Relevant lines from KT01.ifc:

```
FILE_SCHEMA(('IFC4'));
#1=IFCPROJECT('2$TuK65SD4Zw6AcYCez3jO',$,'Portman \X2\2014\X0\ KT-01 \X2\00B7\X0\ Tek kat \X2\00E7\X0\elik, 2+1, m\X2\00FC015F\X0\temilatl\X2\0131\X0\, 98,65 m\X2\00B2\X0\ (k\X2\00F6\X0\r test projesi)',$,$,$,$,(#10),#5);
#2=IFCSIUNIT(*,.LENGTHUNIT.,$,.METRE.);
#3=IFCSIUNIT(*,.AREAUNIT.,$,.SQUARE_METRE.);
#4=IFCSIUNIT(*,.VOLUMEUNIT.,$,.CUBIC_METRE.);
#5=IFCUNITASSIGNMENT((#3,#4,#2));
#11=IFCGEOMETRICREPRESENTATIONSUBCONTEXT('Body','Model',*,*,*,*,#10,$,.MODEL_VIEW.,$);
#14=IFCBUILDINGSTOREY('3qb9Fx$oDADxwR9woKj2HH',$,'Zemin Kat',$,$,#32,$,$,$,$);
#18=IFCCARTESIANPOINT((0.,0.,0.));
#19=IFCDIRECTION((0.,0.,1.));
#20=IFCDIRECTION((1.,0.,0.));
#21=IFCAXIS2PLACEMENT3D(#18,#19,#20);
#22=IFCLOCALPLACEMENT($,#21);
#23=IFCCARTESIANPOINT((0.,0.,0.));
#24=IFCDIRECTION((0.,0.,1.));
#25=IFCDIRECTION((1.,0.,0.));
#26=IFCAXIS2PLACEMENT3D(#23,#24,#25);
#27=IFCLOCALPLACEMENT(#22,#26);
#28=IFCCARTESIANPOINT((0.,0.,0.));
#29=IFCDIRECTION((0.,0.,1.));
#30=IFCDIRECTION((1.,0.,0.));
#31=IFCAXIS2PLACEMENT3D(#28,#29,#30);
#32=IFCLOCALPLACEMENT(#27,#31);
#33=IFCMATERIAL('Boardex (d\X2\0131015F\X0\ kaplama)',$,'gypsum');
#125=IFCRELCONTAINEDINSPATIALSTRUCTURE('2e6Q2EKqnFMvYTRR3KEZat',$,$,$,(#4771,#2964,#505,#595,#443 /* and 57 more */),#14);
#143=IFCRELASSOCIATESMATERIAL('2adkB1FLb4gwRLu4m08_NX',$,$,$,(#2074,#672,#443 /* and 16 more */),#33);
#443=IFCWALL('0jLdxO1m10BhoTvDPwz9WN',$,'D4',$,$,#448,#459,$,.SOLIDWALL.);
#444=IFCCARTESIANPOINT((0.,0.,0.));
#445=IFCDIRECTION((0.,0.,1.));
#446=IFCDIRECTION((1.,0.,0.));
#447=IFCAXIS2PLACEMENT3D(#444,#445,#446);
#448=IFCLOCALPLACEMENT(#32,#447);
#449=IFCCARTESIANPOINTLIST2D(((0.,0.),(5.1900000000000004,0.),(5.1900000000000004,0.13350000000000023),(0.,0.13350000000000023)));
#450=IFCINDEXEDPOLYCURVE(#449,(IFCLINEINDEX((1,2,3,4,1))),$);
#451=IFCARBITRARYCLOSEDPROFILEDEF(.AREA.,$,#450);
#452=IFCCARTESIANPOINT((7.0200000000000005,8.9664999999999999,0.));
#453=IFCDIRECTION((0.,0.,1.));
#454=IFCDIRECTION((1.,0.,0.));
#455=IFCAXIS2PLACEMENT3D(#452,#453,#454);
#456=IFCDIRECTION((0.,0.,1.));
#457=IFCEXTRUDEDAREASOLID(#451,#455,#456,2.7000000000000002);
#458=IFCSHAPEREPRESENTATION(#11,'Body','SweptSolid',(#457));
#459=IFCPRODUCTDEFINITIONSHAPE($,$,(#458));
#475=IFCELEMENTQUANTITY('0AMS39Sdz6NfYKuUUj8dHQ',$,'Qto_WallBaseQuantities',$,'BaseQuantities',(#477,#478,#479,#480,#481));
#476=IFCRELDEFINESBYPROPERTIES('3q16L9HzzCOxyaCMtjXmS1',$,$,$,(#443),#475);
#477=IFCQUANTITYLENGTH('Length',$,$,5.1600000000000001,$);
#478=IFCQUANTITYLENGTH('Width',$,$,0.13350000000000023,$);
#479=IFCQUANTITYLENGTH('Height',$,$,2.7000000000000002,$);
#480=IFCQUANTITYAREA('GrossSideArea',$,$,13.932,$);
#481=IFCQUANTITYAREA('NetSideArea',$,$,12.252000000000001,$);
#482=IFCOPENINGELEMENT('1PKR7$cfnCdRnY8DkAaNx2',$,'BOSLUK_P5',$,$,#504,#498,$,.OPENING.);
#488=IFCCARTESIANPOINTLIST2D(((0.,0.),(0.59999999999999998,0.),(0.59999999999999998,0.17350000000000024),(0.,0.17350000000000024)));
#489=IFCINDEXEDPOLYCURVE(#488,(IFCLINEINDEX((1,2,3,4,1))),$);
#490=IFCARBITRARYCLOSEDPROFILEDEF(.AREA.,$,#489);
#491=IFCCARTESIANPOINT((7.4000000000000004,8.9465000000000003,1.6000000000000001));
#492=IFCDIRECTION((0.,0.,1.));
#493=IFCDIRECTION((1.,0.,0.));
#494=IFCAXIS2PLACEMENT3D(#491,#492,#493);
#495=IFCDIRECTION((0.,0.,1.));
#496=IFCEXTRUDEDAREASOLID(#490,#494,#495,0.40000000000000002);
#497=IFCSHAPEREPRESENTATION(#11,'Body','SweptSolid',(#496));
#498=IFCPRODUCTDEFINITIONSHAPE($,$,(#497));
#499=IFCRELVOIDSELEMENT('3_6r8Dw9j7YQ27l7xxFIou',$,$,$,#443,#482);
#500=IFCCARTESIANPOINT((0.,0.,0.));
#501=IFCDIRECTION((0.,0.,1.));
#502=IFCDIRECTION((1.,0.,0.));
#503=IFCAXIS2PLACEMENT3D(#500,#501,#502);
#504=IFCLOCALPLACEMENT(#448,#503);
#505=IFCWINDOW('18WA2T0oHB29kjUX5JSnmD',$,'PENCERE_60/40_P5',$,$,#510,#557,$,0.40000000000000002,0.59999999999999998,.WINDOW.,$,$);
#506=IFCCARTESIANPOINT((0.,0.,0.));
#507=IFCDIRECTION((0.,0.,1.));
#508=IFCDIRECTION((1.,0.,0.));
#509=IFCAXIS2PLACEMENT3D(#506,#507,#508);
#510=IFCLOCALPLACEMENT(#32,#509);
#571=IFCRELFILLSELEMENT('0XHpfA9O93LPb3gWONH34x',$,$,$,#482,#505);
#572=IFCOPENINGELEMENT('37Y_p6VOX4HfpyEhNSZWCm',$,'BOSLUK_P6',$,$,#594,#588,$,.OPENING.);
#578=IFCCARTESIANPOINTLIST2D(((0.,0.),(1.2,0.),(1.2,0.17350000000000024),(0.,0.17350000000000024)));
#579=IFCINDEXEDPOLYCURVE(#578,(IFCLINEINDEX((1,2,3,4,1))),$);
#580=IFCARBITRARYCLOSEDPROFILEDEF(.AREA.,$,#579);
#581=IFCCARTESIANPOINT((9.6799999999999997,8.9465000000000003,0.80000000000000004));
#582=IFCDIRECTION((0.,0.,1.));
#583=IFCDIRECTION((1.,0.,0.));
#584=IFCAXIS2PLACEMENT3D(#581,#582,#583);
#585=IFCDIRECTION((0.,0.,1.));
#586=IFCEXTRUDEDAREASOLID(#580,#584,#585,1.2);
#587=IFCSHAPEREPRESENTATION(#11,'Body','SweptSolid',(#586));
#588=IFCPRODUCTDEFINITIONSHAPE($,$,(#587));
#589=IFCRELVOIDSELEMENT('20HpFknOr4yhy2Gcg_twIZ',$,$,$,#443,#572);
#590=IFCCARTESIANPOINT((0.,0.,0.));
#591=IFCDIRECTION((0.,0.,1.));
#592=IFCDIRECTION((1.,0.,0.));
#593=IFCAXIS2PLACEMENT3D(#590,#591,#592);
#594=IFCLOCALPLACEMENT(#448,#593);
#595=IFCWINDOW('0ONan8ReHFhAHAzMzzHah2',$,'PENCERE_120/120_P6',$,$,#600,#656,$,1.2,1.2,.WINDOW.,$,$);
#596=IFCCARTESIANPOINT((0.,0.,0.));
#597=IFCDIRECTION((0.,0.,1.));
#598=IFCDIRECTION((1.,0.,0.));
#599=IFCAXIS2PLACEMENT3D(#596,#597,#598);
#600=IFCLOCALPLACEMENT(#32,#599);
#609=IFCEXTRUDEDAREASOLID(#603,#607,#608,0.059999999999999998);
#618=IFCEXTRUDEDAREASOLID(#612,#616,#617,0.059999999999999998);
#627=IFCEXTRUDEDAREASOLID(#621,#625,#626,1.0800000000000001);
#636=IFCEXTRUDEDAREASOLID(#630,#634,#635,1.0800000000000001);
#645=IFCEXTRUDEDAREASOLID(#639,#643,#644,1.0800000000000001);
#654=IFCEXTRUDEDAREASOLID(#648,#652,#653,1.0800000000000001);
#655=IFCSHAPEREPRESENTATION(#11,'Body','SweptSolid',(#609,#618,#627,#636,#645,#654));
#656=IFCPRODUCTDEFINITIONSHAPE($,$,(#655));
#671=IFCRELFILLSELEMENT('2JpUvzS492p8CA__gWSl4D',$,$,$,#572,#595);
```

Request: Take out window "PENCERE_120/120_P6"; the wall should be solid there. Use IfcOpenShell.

```python
import ifcopenshell
import ifcopenshell.api.feature
import ifcopenshell.api.pset
import ifcopenshell.api.root
import ifcopenshell.geom
import ifcopenshell.util.element
import ifcopenshell.util.shape
import ifcopenshell.util.unit

model = ifcopenshell.open("KT01.ifc")
area_scale = ifcopenshell.util.unit.calculate_unit_scale(model, "AREAUNIT")
settings = ifcopenshell.geom.settings()


def volume(element):
    """Net volume in cubic metres, openings subtracted."""
    shape = ifcopenshell.geom.create_shape(settings, element)
    return ifcopenshell.util.shape.get_volume(shape.geometry)


window = model.by_guid("0ONan8ReHFhAHAzMzzHah2")
opening = window.FillsVoids[0].RelatingOpeningElement
wall = opening.VoidsElements[0].RelatingBuildingElement
before = volume(wall)

ifcopenshell.api.root.remove_product(model, product=window)
ifcopenshell.api.feature.remove_feature(model, feature=opening)

after = volume(wall)
thickness = 0.1335  # wall thickness in metres

# Update the wall's stored quantities.
qto = model.by_id(ifcopenshell.util.element.get_pset(wall, "Qto_WallBaseQuantities", should_inherit=False)["id"])
ifcopenshell.api.pset.edit_qto(model, qto=qto, properties={"NetSideArea": after / thickness / area_scale})

print(f"wall volume {before:.3f} -> {after:.3f} m3")

model.write("KT01_edited.ifc")
```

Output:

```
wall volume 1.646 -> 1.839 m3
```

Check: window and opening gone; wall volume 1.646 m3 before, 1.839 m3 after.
